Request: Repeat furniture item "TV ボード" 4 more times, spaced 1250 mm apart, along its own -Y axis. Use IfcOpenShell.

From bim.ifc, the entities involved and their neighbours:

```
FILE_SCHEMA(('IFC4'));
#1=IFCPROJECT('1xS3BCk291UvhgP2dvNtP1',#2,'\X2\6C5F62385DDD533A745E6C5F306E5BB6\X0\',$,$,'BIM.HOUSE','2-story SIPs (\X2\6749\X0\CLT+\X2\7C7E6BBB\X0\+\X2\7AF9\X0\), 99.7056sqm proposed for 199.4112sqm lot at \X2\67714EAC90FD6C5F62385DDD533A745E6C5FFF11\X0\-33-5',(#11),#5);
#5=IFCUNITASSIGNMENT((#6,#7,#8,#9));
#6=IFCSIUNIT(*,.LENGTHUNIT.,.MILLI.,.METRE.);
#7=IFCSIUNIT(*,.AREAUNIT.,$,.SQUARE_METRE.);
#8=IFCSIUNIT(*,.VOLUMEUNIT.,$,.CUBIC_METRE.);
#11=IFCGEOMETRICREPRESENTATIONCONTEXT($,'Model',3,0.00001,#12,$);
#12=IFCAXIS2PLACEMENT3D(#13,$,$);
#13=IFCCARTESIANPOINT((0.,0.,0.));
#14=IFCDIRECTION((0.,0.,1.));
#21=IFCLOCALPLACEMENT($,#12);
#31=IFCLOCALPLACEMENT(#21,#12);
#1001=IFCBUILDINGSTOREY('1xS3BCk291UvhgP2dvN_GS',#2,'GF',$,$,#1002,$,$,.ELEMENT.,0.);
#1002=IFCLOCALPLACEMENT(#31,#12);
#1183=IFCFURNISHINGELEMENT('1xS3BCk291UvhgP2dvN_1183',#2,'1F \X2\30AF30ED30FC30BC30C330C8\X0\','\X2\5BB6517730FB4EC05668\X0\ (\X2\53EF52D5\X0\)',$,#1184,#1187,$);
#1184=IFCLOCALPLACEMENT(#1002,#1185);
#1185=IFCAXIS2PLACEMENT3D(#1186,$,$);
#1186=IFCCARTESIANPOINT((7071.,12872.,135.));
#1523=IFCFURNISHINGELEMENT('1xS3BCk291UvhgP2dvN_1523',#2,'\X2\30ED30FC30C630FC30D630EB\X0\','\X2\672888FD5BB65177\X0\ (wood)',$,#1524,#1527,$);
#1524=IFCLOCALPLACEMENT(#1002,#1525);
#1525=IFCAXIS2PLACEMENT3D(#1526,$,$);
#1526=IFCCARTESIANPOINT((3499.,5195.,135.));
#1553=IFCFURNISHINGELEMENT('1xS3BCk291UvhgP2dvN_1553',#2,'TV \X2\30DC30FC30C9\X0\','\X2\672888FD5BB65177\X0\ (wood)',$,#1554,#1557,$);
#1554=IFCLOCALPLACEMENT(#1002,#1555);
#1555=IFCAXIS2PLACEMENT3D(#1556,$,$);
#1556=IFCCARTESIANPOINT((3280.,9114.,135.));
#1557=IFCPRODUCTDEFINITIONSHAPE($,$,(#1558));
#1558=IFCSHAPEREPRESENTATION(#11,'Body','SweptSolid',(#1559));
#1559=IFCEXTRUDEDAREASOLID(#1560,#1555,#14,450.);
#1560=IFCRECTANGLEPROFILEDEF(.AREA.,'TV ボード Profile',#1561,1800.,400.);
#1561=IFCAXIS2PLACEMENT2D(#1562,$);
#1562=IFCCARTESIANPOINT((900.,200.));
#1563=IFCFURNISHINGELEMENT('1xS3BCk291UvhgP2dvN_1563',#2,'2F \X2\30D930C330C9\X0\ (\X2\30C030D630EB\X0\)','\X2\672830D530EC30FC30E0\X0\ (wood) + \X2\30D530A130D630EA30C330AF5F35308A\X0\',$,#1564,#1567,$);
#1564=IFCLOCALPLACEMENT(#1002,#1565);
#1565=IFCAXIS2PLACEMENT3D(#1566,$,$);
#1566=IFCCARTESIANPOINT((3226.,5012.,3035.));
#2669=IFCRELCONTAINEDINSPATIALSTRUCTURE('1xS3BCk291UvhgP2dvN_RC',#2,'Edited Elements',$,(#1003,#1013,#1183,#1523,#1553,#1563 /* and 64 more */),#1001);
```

```python
import ifcopenshell
import ifcopenshell.api.geometry
import ifcopenshell.api.root
import ifcopenshell.util.element
import ifcopenshell.util.placement

model = ifcopenshell.open("bim.ifc")


def reuse_history(source, copy):
    """copy_class also copies each property set's owner history, people and application; keep the originals."""
    for rel in copy.IsDefinedBy:
        if rel.is_a("IfcRelDefinesByProperties") and (history := rel.RelatingPropertyDefinition.OwnerHistory):
            rel.RelatingPropertyDefinition.OwnerHistory = source.OwnerHistory
            ifcopenshell.util.element.remove_deep2(model, history)


source = model.by_id(1553)
base = ifcopenshell.util.placement.get_local_placement(source.ObjectPlacement)
step = -base[:3, 1] * 1250.0

for i in range(1, 5):
    copy = ifcopenshell.api.root.copy_class(model, product=source)
    copy.Representation = ifcopenshell.util.element.copy_deep(
        model, source.Representation, exclude=["IfcGeometricRepresentationContext", "IfcRepresentationMap"]
    )
    reuse_history(source, copy)
    matrix = base.copy()
    matrix[:3, 3] += i * step
    print("added at", matrix[:3, 3].round(3) + 0.0)
    ifcopenshell.api.geometry.edit_object_placement(model, product=copy, matrix=matrix, is_si=False)

model.write("bim_rev.ifc")
```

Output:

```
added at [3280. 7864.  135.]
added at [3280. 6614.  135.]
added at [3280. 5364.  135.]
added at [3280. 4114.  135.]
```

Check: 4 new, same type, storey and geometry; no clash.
